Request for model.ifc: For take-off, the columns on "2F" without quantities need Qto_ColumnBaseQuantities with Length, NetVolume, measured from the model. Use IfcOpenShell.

First a look at what the model holds.

```python
import ifcopenshell
import ifcopenshell.util.element
import ifcopenshell.util.unit

model = ifcopenshell.open("model.ifc")
print(model.schema)
for unit_type in ("LENGTHUNIT", "AREAUNIT", "VOLUMEUNIT"):
    print(unit_type, ifcopenshell.util.unit.calculate_unit_scale(model, unit_type))
storey = next(s for s in model.by_type("IfcBuildingStorey") if s.Name == "2F")
columns = [e for e in ifcopenshell.util.element.get_decomposition(storey) if e.is_a("IfcColumn")]
for e in sorted(columns, key=lambda e: e.id()):
    print(e.id(), e.is_a(), e.Name, list(ifcopenshell.util.element.get_psets(e, qtos_only=True)), sep=" | ")
```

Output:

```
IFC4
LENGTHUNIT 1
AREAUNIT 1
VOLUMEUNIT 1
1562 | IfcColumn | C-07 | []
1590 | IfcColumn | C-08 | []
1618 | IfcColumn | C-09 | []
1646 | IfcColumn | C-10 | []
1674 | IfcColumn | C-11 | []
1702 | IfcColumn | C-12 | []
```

```python
import ifcopenshell
import ifcopenshell.api.pset
import ifcopenshell.geom
import ifcopenshell.util.element
import ifcopenshell.util.shape
import ifcopenshell.util.unit

model = ifcopenshell.open("model.ifc")
unit_scale = ifcopenshell.util.unit.calculate_unit_scale(model)
volume_scale = ifcopenshell.util.unit.calculate_unit_scale(model, "VOLUMEUNIT")
settings = ifcopenshell.geom.settings()

storey = next(s for s in model.by_type("IfcBuildingStorey") if s.Name == "2F")
columns = [e for e in ifcopenshell.util.element.get_decomposition(storey) if e.is_a("IfcColumn")]

for e in sorted(columns, key=lambda e: e.id()):
    if ifcopenshell.util.element.get_psets(e, qtos_only=True, should_inherit=False):
        continue
    # Geometry comes back in metres, in the element's own axes.
    shape = ifcopenshell.geom.create_shape(settings, e)
    values = {
        "Length": ifcopenshell.util.shape.get_z(shape.geometry) / unit_scale,
        "NetVolume": ifcopenshell.util.shape.get_volume(shape.geometry) / volume_scale,
    }
    qto = ifcopenshell.api.pset.add_qto(model, product=e, name="Qto_ColumnBaseQuantities")
    ifcopenshell.api.pset.edit_qto(model, qto=qto, properties=values)
    print(e.id(), {k: round(v, 3) for k, v in values.items()})

model.write("model-out.ifc")
```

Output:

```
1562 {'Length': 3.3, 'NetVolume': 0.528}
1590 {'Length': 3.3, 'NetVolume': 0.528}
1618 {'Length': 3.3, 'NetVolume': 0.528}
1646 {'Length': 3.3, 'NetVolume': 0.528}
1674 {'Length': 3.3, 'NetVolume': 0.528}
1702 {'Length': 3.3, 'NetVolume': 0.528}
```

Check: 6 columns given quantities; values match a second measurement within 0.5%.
